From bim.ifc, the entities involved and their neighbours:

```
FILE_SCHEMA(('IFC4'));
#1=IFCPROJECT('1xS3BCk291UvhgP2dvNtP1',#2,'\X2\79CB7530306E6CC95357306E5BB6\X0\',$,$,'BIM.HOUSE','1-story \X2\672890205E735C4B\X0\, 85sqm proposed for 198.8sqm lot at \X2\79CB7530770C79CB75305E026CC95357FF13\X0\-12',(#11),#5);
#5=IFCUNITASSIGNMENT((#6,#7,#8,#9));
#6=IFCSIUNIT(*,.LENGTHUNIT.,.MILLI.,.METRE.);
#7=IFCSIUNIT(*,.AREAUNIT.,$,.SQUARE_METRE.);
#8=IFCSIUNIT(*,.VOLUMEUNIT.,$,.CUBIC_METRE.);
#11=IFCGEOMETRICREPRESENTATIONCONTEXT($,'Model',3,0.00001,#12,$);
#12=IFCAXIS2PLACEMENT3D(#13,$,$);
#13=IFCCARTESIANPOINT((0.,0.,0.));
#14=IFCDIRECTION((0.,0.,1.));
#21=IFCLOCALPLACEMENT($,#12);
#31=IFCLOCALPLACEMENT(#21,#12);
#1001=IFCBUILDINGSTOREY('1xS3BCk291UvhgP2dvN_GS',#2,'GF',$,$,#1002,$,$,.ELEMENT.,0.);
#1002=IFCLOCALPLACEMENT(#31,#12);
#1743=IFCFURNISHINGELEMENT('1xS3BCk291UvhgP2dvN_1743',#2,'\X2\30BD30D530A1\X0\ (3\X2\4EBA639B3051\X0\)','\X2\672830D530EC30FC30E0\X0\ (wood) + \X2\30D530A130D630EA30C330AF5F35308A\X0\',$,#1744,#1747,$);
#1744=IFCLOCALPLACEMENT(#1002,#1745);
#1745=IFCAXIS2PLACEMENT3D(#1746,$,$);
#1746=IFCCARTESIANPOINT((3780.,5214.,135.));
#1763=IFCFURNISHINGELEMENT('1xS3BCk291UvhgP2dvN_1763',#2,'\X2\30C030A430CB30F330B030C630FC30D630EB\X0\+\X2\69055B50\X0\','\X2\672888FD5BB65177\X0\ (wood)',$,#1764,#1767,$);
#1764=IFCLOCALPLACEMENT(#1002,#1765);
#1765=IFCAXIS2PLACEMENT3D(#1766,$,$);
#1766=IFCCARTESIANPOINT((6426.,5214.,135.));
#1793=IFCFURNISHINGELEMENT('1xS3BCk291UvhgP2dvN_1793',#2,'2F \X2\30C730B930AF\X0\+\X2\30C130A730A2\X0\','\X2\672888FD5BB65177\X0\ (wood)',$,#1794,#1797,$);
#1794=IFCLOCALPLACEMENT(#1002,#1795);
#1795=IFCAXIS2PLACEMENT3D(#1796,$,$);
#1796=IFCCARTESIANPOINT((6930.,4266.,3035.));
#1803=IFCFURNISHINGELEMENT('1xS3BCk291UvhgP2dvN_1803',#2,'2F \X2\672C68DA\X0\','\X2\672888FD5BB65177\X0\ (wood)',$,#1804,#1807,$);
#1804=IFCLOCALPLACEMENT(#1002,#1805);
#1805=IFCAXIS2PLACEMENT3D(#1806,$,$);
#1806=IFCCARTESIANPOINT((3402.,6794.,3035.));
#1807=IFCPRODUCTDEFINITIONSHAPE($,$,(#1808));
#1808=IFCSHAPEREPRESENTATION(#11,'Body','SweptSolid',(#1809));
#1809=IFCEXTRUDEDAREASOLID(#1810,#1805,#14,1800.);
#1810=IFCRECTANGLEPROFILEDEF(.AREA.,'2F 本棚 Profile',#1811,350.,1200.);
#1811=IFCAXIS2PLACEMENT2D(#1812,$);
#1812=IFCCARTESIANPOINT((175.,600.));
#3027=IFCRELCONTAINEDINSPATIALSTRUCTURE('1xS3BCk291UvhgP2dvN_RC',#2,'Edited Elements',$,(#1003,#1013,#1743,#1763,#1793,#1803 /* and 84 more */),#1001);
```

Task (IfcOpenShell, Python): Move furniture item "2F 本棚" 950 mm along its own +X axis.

```python
import ifcopenshell
import ifcopenshell.api.geometry
import ifcopenshell.util.placement

model = ifcopenshell.open("bim.ifc")

item = model.by_guid("1xS3BCk291UvhgP2dvN_1803")
matrix = ifcopenshell.util.placement.get_local_placement(item.ObjectPlacement)
matrix[:3, 3] += matrix[:3, 0] * 950.0
ifcopenshell.api.geometry.edit_object_placement(model, product=item, matrix=matrix, is_si=False)

print(ifcopenshell.util.placement.get_local_placement(item.ObjectPlacement).round(3) + 0.0)

model.write("bim_v2.ifc")
```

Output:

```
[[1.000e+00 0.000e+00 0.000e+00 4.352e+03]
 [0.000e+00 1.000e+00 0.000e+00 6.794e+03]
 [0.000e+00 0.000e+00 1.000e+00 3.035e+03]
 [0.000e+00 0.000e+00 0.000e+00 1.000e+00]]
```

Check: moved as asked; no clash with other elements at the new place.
